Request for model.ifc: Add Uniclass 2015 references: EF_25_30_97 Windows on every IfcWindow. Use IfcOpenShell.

First a look at what the model holds.

```python
import ifcopenshell

model = ifcopenshell.open("model.ifc")
print(model.schema)
print("classifications:", [c.Name for c in model.by_type("IfcClassification")])
for ifc_class in ("IfcDoor", "IfcRoof", "IfcStair", "IfcWall", "IfcWindow"):
    print(ifc_class, len(model.by_type(ifc_class)))
```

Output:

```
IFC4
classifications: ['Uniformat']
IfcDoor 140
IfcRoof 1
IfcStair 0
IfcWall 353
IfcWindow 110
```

```python
import ifcopenshell
import ifcopenshell.api.classification

model = ifcopenshell.open("model.ifc")

system = ifcopenshell.api.classification.add_classification(model, classification="Uniclass 2015")

codes = {
    "IfcWindow": ("EF_25_30_97", "Windows"),
}
for ifc_class, (code, name) in codes.items():
    products = model.by_type(ifc_class)
    ifcopenshell.api.classification.add_reference(
        model, products=products, classification=system, identification=code, name=name
    )
    print(code, len(products))

model.write("model-out.ifc")
```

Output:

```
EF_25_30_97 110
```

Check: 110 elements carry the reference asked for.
